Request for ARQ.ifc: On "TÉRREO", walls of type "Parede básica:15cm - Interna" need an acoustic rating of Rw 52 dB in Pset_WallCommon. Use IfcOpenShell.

First a look at what the model holds.

```python
import ifcopenshell
import ifcopenshell.util.element

model = ifcopenshell.open("ARQ.ifc")
print(model.schema)
storey = next(s for s in model.by_type("IfcBuildingStorey") if s.Name == "TÉRREO")
walls = [e for e in ifcopenshell.util.element.get_decomposition(storey) if e.is_a("IfcWall")]
seen = {}
for e in walls:
    element_type = ifcopenshell.util.element.get_type(e)
    key = (element_type.Name if element_type != e and element_type else None, ifcopenshell.util.element.get_pset(e, "Pset_WallCommon", "AcousticRating"))
    seen[key] = seen.get(key, 0) + 1
for (name, value), count in sorted(seen.items(), key=str):
    print(count, "x", name, "|", value)
```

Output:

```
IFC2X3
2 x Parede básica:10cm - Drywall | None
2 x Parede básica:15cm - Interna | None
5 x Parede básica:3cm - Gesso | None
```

```python
import ifcopenshell
import ifcopenshell.api.pset
import ifcopenshell.util.element

model = ifcopenshell.open("ARQ.ifc")

storey = next(s for s in model.by_type("IfcBuildingStorey") if s.Name == "TÉRREO")
walls = [e for e in ifcopenshell.util.element.get_decomposition(storey) if e.is_a("IfcWall")]

count = 0
for e in walls:
    element_type = ifcopenshell.util.element.get_type(e)
    if element_type in (None, e) or element_type.Name != "Parede básica:15cm - Interna":
        continue
    # add_pset returns the element's existing set when there is one.
    pset = ifcopenshell.api.pset.add_pset(model, product=e, name="Pset_WallCommon")
    ifcopenshell.api.pset.edit_pset(model, pset=pset, properties={"AcousticRating": "Rw 52 dB"})
    count += 1

print(count, "walls updated")

model.write("ARQ_v2.ifc")
```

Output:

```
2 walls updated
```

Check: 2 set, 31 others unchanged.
